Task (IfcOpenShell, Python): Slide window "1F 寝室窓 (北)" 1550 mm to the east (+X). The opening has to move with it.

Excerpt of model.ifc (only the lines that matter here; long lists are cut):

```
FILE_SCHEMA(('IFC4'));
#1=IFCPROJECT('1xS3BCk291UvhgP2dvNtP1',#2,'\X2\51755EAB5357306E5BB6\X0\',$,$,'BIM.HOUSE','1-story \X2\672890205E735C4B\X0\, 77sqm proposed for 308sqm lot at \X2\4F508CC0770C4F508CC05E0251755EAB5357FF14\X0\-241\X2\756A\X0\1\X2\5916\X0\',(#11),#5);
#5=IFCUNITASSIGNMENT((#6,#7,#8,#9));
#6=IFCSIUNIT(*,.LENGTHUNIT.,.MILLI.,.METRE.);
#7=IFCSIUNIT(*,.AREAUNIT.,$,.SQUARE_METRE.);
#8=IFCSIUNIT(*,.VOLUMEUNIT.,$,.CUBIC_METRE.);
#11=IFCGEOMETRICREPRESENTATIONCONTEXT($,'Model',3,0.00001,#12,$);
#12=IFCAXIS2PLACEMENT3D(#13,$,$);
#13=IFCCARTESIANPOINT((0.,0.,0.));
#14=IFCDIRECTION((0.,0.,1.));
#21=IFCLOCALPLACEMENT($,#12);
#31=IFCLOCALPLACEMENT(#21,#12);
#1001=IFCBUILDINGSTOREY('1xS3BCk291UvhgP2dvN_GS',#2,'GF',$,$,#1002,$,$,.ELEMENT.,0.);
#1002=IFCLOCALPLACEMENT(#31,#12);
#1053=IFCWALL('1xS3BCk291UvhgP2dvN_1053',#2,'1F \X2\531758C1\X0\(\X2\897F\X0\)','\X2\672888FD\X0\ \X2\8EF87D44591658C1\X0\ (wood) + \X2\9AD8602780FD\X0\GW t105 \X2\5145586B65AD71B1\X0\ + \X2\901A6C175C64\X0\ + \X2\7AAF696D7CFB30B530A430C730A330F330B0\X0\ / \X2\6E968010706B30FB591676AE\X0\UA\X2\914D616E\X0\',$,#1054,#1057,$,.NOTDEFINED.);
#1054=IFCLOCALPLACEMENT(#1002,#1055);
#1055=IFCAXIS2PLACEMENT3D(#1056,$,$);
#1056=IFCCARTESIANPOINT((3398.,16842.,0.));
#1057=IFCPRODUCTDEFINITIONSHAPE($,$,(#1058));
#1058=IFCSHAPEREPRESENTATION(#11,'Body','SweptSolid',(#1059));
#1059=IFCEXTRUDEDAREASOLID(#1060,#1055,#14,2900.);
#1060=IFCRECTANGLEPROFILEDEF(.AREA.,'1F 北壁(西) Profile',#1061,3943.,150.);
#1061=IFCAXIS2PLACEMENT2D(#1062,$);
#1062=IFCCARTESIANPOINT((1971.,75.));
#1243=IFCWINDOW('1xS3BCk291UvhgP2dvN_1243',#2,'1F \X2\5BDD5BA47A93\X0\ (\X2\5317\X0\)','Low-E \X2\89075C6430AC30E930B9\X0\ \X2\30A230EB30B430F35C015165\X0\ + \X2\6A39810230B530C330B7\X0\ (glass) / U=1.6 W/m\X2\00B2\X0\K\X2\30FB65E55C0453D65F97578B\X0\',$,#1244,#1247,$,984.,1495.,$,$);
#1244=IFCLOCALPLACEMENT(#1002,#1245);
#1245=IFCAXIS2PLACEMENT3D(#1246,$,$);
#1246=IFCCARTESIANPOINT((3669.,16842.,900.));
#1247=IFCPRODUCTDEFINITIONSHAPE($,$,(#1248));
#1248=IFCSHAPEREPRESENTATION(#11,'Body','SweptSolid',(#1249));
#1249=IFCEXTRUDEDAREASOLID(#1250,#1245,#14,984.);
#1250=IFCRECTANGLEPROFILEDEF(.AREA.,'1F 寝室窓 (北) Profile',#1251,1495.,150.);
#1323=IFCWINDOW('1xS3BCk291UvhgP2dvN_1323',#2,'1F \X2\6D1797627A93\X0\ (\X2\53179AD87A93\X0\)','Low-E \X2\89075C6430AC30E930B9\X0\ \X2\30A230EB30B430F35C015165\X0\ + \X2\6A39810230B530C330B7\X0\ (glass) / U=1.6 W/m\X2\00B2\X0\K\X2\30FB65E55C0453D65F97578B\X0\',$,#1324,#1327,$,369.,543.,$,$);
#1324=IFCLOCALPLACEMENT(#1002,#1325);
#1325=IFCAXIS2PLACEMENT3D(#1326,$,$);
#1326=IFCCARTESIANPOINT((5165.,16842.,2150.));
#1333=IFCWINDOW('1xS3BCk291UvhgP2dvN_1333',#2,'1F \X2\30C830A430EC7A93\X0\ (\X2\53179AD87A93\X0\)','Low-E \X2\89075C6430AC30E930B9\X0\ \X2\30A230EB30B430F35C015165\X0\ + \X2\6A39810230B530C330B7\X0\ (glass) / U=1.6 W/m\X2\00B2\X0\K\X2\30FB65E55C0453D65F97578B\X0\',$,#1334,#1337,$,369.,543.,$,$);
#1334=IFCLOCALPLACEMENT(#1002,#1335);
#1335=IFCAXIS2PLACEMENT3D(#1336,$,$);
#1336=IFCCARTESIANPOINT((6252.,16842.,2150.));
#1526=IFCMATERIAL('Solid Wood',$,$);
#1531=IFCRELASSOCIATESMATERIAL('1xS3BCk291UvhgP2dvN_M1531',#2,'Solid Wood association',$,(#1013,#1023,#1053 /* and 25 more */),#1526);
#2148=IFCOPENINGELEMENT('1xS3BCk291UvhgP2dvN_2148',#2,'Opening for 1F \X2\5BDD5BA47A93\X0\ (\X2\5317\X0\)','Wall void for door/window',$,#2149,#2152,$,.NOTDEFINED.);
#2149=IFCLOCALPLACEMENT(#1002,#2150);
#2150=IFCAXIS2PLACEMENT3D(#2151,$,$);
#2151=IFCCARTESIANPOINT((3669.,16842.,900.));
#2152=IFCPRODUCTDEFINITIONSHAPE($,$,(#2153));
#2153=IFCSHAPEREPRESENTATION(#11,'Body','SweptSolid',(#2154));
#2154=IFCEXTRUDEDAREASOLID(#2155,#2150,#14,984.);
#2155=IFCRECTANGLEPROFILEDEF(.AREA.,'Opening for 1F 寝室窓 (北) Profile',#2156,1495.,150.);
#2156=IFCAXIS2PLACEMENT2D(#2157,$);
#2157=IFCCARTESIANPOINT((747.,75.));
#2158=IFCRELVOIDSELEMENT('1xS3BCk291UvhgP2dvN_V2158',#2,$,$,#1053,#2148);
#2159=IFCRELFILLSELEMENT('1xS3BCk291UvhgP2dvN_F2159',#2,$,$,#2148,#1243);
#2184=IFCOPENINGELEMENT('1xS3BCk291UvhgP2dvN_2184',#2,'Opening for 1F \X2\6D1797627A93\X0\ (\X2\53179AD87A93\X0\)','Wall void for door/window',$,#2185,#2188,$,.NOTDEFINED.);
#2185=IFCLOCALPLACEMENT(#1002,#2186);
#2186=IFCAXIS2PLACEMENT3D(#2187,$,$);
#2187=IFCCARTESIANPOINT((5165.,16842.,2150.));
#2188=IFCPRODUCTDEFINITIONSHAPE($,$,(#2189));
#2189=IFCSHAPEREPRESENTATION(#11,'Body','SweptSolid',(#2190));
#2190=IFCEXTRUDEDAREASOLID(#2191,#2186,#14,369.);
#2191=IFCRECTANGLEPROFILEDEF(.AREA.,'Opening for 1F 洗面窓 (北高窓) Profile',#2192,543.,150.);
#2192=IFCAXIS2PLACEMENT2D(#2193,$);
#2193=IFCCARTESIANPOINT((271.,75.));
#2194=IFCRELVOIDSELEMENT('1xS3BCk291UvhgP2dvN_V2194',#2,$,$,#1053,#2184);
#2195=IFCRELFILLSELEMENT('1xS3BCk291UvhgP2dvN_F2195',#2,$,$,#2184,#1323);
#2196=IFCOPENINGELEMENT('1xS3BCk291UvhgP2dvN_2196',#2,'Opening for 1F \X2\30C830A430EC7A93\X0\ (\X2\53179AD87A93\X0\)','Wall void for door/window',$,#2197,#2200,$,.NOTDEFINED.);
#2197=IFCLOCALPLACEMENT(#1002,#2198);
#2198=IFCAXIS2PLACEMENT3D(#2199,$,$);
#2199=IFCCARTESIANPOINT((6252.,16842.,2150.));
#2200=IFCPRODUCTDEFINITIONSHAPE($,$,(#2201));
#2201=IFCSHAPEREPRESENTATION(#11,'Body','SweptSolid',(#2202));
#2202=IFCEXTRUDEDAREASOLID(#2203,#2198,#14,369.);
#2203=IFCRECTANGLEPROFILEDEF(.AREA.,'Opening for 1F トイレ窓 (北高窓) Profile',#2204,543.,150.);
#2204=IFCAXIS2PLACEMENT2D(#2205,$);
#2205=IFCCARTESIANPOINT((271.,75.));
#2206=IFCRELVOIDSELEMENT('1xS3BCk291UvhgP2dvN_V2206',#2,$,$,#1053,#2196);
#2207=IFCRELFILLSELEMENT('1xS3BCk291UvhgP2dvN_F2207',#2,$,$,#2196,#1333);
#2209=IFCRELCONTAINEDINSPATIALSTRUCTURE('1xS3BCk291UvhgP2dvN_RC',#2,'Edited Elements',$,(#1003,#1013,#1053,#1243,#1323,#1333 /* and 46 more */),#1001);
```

```python
import ifcopenshell
import ifcopenshell.api.geometry
import ifcopenshell.util.placement

model = ifcopenshell.open("model.ifc")

window = model.by_guid("1xS3BCk291UvhgP2dvN_1243")
opening = window.FillsVoids[0].RelatingOpeningElement
wall = opening.VoidsElements[0].RelatingBuildingElement

wall_matrix = ifcopenshell.util.placement.get_local_placement(wall.ObjectPlacement)
shift = wall_matrix[:3, 0] * 1550.0
before = ifcopenshell.util.placement.get_local_placement(window.ObjectPlacement)[:3, 3].copy()

# The window is not placed relative to its opening, so move both.
for product in (opening, window):
    matrix = ifcopenshell.util.placement.get_local_placement(product.ObjectPlacement)
    matrix[:3, 3] += shift
    ifcopenshell.api.geometry.edit_object_placement(model, product=product, matrix=matrix, is_si=False)

after = ifcopenshell.util.placement.get_local_placement(window.ObjectPlacement)[:3, 3]
print("window moved by", (after - before).round(3) + 0.0)

model.write("model_updated.ifc")
```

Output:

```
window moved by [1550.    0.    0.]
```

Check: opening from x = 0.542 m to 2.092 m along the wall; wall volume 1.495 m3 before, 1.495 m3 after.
